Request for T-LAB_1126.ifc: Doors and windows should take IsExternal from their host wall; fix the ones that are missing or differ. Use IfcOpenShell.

First a look at what the model holds.

```python
import ifcopenshell
import ifcopenshell.util.element

model = ifcopenshell.open("T-LAB_1126.ifc")
print(model.schema)
seen = {}
for e in model.by_type("IfcDoor") + model.by_type("IfcWindow"):
    if not e.FillsVoids:
        continue
    host = e.FillsVoids[0].RelatingOpeningElement.VoidsElements[0].RelatingBuildingElement
    own = ifcopenshell.util.element.get_pset(e, f"Pset_{e.is_a()[3:].removesuffix('StandardCase')}Common", "IsExternal")
    wall = ifcopenshell.util.element.get_pset(host, "Pset_WallCommon", "IsExternal")
    seen[e.is_a(), own, wall] = seen.get((e.is_a(), own, wall), 0) + 1
for (cls, own, wall), count in sorted(seen.items(), key=str):
    print(count, cls, "IsExternal:", own, "| host wall:", wall)
```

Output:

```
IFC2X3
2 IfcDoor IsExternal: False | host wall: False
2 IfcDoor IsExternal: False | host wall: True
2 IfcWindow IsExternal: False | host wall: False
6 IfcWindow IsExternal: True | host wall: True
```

```python
import ifcopenshell
import ifcopenshell.api.pset
import ifcopenshell.util.element

model = ifcopenshell.open("T-LAB_1126.ifc")

count = 0
for ifc_class, pset_name in (("IfcDoor", "Pset_DoorCommon"), ("IfcWindow", "Pset_WindowCommon")):
    for e in model.by_type(ifc_class):
        if not e.FillsVoids:
            continue
        host = e.FillsVoids[0].RelatingOpeningElement.VoidsElements[0].RelatingBuildingElement
        external = ifcopenshell.util.element.get_pset(host, "Pset_WallCommon", "IsExternal")
        if external is None or ifcopenshell.util.element.get_pset(e, pset_name, "IsExternal") == external:
            continue
        pset = ifcopenshell.api.pset.add_pset(model, product=e, name=pset_name)
        ifcopenshell.api.pset.edit_pset(model, pset=pset, properties={"IsExternal": external})
        count += 1

print(count, "updated")

model.write("T-LAB_1126_v2.ifc")
```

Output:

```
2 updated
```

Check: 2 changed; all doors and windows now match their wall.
